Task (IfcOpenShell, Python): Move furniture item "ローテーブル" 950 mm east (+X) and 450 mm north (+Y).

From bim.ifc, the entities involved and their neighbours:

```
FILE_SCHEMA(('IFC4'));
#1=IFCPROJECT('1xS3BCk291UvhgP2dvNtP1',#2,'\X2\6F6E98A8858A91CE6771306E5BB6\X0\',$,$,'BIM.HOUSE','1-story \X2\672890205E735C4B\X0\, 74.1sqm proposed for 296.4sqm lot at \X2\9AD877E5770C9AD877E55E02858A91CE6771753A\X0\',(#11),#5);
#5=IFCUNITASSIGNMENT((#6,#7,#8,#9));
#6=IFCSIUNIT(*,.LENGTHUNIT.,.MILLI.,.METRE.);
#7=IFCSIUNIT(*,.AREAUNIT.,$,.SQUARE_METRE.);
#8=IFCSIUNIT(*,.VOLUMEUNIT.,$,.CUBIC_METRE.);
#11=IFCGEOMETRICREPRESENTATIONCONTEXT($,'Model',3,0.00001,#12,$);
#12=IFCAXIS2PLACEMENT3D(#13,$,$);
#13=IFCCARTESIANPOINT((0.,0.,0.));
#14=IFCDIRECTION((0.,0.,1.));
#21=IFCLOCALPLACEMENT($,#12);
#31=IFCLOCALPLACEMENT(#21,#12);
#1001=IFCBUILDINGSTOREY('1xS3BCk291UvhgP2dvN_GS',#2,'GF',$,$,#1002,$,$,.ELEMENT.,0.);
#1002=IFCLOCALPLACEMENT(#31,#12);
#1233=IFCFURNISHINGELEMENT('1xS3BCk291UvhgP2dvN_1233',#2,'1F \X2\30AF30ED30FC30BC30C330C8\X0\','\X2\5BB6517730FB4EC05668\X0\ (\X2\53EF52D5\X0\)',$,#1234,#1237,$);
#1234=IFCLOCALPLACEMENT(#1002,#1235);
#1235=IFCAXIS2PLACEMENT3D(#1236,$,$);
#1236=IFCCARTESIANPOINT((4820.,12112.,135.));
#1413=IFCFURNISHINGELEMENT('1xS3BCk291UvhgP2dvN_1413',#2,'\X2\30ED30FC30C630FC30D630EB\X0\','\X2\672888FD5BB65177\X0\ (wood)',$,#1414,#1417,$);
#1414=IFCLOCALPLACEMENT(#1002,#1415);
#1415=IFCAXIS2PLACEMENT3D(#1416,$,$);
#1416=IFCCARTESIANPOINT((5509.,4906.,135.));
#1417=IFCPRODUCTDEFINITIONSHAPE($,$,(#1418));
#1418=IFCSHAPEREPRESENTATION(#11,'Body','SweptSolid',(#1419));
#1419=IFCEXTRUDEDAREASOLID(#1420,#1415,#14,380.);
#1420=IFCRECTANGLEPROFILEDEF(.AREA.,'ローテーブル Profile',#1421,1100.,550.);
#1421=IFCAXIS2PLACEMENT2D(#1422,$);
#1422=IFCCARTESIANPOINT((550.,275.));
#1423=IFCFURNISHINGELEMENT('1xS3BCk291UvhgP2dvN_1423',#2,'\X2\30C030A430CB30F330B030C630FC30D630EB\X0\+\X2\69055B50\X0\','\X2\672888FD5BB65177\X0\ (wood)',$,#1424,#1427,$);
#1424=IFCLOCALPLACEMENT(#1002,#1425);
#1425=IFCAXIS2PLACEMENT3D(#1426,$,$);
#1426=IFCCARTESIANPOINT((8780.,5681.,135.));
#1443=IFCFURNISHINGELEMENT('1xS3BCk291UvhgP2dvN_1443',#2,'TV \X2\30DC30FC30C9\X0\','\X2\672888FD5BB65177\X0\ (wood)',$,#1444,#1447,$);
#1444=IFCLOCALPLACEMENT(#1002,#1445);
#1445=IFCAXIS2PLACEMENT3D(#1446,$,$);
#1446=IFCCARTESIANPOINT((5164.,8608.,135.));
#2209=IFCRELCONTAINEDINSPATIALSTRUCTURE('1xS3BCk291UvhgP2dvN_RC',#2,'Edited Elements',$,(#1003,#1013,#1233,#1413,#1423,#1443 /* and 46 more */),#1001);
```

```python
import ifcopenshell
import ifcopenshell.api.geometry
import ifcopenshell.util.placement

model = ifcopenshell.open("bim.ifc")

item = model.by_id(1413)
matrix = ifcopenshell.util.placement.get_local_placement(item.ObjectPlacement)
matrix[0, 3] += 950.0
matrix[1, 3] += 450.0
ifcopenshell.api.geometry.edit_object_placement(model, product=item, matrix=matrix, is_si=False)

print(ifcopenshell.util.placement.get_local_placement(item.ObjectPlacement).round(3) + 0.0)

model.write("bim_edited.ifc")
```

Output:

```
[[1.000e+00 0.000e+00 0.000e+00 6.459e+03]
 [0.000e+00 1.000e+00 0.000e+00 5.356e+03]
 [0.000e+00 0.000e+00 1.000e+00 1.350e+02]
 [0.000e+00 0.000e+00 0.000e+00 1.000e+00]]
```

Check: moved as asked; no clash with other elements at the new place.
